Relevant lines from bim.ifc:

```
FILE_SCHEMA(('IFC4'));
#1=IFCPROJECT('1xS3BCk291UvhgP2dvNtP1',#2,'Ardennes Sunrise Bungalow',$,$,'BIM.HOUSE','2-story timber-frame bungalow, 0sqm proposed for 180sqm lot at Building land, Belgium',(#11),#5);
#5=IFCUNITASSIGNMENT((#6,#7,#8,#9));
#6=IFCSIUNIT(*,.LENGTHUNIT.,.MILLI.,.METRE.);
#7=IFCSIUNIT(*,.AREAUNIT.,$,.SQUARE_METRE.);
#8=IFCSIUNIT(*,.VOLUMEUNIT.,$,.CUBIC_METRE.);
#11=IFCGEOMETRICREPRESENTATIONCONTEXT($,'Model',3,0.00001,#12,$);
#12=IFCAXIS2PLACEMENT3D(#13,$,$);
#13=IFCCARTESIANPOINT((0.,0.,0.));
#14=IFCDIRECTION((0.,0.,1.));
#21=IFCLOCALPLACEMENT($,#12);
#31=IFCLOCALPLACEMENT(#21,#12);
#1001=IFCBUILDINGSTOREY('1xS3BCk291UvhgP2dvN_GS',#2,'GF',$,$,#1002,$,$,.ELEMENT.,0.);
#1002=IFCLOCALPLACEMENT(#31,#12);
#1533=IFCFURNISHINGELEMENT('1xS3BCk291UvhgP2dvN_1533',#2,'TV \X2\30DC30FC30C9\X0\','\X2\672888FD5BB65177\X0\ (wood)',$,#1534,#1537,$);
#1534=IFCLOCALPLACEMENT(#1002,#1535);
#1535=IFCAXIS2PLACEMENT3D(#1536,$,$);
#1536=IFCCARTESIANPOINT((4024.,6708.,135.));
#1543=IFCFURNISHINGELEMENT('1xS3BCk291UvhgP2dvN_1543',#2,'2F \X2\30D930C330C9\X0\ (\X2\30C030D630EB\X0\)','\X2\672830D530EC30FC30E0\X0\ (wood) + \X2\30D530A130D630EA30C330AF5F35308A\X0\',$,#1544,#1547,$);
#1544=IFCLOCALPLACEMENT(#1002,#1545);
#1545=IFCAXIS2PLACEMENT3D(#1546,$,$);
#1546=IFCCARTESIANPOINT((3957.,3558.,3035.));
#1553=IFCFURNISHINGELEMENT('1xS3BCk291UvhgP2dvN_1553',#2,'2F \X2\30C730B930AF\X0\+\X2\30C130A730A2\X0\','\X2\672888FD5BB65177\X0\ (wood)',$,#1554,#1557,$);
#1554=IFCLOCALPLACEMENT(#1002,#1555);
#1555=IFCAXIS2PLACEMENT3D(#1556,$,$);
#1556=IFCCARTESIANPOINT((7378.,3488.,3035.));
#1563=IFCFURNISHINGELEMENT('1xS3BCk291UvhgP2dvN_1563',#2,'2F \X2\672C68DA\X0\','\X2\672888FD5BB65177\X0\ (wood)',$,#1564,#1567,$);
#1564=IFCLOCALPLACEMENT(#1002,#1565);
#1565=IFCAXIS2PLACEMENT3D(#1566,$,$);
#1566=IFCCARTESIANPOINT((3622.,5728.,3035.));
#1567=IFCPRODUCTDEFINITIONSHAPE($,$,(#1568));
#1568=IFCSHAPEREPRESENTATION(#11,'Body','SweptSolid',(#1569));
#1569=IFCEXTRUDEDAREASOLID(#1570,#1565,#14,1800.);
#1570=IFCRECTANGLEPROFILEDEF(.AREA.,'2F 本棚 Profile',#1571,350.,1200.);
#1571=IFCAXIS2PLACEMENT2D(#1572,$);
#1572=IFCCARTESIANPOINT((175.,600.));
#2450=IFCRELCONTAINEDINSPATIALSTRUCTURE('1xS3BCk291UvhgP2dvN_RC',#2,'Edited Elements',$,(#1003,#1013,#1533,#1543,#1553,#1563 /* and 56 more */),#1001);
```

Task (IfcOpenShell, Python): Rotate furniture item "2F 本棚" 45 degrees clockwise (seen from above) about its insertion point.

```python
import ifcopenshell
import ifcopenshell.api.geometry
import ifcopenshell.util.placement

model = ifcopenshell.open("bim.ifc")

item = model.by_guid("1xS3BCk291UvhgP2dvN_1563")
matrix = ifcopenshell.util.placement.get_local_placement(item.ObjectPlacement)
matrix = matrix @ ifcopenshell.util.placement.rotation(-45, "Z")
ifcopenshell.api.geometry.edit_object_placement(model, product=item, matrix=matrix, is_si=False)

print(ifcopenshell.util.placement.get_local_placement(item.ObjectPlacement).round(3) + 0.0)

model.write("bim_v2.ifc")
```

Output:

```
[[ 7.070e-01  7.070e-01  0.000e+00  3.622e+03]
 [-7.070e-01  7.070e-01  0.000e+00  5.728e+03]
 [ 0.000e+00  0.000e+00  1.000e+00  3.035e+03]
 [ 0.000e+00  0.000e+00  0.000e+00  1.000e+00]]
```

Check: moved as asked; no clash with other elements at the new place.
